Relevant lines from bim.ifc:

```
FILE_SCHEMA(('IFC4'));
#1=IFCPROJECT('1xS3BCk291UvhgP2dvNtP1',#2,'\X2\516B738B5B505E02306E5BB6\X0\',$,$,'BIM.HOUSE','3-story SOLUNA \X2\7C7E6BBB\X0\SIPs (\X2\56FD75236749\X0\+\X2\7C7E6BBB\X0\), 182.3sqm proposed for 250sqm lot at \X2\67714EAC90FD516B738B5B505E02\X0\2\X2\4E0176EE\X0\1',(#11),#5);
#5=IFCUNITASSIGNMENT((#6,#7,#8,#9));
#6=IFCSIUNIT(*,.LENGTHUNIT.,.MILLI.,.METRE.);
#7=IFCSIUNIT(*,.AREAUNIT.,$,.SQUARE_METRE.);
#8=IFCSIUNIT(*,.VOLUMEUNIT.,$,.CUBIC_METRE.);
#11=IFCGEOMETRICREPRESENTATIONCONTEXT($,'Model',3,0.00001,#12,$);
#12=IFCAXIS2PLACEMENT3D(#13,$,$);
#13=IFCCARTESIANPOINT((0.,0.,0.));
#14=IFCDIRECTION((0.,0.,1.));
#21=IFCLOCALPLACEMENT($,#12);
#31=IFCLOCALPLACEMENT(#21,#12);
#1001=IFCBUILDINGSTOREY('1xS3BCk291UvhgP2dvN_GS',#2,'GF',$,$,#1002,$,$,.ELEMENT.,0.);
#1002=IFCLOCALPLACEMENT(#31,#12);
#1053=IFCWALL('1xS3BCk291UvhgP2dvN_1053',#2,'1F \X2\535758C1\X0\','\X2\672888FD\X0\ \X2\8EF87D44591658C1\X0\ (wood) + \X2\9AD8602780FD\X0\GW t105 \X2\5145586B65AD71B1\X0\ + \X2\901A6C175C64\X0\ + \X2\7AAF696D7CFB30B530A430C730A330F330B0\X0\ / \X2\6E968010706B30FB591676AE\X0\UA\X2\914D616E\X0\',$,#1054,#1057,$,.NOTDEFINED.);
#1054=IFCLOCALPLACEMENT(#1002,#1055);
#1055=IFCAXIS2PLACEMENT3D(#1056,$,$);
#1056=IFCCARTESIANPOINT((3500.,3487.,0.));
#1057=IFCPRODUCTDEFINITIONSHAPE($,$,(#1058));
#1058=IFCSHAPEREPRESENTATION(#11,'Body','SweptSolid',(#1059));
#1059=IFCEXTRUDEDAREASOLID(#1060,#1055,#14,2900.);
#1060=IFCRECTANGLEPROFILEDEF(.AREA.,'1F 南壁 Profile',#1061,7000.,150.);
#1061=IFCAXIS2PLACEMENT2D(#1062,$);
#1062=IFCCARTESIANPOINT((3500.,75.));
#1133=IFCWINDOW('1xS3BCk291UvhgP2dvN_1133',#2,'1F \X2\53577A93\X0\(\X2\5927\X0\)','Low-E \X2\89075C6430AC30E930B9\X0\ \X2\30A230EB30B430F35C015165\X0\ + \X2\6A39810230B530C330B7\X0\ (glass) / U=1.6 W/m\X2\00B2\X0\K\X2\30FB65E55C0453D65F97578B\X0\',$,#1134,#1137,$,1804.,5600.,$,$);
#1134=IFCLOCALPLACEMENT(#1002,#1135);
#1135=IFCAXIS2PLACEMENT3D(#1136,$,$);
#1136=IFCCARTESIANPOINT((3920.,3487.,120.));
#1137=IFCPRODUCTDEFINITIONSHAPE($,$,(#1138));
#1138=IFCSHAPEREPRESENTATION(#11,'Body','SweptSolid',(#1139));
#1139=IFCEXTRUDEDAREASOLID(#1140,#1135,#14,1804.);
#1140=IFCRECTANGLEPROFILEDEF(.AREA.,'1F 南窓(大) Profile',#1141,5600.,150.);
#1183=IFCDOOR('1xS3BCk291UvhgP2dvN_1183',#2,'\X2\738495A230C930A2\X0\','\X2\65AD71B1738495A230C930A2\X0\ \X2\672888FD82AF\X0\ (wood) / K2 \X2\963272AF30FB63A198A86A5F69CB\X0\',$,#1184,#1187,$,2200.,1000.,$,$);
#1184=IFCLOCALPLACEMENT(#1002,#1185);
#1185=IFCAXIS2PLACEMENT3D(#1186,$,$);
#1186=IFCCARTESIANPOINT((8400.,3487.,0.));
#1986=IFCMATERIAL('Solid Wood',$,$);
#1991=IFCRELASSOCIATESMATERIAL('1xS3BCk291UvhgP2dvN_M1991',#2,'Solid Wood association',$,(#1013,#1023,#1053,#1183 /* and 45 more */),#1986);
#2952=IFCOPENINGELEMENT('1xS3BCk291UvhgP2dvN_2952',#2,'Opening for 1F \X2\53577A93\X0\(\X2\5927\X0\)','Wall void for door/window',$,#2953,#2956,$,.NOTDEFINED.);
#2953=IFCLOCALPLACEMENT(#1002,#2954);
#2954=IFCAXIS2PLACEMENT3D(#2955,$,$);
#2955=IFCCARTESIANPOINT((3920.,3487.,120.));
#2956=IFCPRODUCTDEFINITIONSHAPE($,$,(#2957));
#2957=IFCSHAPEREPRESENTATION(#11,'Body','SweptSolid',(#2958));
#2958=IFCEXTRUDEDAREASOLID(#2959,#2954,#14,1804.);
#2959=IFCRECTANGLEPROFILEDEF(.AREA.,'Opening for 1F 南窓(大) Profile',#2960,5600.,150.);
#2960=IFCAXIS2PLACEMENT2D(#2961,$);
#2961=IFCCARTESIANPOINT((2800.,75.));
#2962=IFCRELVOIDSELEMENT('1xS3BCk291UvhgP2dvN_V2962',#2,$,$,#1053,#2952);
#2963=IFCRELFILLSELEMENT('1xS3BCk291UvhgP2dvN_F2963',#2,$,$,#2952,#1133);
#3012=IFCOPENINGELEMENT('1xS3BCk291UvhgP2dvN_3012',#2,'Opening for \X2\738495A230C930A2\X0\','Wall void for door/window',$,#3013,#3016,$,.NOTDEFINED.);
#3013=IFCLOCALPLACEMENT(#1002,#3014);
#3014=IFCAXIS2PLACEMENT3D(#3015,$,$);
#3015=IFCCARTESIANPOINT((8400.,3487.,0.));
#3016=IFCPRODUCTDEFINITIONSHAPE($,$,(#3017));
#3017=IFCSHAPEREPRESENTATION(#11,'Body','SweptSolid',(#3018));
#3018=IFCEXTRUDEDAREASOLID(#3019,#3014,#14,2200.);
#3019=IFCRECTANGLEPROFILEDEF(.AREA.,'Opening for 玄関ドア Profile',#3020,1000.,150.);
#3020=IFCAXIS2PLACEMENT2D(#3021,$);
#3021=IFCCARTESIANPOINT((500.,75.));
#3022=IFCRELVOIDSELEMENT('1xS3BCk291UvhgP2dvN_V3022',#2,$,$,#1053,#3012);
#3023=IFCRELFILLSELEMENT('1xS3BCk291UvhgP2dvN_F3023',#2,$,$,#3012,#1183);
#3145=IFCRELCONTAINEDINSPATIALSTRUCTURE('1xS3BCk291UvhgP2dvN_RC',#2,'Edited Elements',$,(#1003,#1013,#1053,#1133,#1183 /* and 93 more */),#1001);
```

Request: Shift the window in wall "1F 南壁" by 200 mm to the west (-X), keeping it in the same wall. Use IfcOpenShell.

```python
import ifcopenshell
import ifcopenshell.api.geometry
import ifcopenshell.util.placement
import ifcopenshell.util.unit

model = ifcopenshell.open("bim.ifc")
unit_scale = ifcopenshell.util.unit.calculate_unit_scale(model)

window = model.by_guid("1xS3BCk291UvhgP2dvN_1133")
opening = window.FillsVoids[0].RelatingOpeningElement
wall = opening.VoidsElements[0].RelatingBuildingElement

wall_matrix = ifcopenshell.util.placement.get_local_placement(wall.ObjectPlacement)
shift = wall_matrix[:3, 0] * -0.2 / unit_scale
before = ifcopenshell.util.placement.get_local_placement(window.ObjectPlacement)[:3, 3].copy()

# The window is not placed relative to its opening, so move both.
for product in (opening, window):
    matrix = ifcopenshell.util.placement.get_local_placement(product.ObjectPlacement)
    matrix[:3, 3] += shift
    ifcopenshell.api.geometry.edit_object_placement(model, product=product, matrix=matrix, is_si=False)

after = ifcopenshell.util.placement.get_local_placement(window.ObjectPlacement)[:3, 3]
print("window moved by", (after - before).round(3) + 0.0)

model.write("bim_rev.ifc")
```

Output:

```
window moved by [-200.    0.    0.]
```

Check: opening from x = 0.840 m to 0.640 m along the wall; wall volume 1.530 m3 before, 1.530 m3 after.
